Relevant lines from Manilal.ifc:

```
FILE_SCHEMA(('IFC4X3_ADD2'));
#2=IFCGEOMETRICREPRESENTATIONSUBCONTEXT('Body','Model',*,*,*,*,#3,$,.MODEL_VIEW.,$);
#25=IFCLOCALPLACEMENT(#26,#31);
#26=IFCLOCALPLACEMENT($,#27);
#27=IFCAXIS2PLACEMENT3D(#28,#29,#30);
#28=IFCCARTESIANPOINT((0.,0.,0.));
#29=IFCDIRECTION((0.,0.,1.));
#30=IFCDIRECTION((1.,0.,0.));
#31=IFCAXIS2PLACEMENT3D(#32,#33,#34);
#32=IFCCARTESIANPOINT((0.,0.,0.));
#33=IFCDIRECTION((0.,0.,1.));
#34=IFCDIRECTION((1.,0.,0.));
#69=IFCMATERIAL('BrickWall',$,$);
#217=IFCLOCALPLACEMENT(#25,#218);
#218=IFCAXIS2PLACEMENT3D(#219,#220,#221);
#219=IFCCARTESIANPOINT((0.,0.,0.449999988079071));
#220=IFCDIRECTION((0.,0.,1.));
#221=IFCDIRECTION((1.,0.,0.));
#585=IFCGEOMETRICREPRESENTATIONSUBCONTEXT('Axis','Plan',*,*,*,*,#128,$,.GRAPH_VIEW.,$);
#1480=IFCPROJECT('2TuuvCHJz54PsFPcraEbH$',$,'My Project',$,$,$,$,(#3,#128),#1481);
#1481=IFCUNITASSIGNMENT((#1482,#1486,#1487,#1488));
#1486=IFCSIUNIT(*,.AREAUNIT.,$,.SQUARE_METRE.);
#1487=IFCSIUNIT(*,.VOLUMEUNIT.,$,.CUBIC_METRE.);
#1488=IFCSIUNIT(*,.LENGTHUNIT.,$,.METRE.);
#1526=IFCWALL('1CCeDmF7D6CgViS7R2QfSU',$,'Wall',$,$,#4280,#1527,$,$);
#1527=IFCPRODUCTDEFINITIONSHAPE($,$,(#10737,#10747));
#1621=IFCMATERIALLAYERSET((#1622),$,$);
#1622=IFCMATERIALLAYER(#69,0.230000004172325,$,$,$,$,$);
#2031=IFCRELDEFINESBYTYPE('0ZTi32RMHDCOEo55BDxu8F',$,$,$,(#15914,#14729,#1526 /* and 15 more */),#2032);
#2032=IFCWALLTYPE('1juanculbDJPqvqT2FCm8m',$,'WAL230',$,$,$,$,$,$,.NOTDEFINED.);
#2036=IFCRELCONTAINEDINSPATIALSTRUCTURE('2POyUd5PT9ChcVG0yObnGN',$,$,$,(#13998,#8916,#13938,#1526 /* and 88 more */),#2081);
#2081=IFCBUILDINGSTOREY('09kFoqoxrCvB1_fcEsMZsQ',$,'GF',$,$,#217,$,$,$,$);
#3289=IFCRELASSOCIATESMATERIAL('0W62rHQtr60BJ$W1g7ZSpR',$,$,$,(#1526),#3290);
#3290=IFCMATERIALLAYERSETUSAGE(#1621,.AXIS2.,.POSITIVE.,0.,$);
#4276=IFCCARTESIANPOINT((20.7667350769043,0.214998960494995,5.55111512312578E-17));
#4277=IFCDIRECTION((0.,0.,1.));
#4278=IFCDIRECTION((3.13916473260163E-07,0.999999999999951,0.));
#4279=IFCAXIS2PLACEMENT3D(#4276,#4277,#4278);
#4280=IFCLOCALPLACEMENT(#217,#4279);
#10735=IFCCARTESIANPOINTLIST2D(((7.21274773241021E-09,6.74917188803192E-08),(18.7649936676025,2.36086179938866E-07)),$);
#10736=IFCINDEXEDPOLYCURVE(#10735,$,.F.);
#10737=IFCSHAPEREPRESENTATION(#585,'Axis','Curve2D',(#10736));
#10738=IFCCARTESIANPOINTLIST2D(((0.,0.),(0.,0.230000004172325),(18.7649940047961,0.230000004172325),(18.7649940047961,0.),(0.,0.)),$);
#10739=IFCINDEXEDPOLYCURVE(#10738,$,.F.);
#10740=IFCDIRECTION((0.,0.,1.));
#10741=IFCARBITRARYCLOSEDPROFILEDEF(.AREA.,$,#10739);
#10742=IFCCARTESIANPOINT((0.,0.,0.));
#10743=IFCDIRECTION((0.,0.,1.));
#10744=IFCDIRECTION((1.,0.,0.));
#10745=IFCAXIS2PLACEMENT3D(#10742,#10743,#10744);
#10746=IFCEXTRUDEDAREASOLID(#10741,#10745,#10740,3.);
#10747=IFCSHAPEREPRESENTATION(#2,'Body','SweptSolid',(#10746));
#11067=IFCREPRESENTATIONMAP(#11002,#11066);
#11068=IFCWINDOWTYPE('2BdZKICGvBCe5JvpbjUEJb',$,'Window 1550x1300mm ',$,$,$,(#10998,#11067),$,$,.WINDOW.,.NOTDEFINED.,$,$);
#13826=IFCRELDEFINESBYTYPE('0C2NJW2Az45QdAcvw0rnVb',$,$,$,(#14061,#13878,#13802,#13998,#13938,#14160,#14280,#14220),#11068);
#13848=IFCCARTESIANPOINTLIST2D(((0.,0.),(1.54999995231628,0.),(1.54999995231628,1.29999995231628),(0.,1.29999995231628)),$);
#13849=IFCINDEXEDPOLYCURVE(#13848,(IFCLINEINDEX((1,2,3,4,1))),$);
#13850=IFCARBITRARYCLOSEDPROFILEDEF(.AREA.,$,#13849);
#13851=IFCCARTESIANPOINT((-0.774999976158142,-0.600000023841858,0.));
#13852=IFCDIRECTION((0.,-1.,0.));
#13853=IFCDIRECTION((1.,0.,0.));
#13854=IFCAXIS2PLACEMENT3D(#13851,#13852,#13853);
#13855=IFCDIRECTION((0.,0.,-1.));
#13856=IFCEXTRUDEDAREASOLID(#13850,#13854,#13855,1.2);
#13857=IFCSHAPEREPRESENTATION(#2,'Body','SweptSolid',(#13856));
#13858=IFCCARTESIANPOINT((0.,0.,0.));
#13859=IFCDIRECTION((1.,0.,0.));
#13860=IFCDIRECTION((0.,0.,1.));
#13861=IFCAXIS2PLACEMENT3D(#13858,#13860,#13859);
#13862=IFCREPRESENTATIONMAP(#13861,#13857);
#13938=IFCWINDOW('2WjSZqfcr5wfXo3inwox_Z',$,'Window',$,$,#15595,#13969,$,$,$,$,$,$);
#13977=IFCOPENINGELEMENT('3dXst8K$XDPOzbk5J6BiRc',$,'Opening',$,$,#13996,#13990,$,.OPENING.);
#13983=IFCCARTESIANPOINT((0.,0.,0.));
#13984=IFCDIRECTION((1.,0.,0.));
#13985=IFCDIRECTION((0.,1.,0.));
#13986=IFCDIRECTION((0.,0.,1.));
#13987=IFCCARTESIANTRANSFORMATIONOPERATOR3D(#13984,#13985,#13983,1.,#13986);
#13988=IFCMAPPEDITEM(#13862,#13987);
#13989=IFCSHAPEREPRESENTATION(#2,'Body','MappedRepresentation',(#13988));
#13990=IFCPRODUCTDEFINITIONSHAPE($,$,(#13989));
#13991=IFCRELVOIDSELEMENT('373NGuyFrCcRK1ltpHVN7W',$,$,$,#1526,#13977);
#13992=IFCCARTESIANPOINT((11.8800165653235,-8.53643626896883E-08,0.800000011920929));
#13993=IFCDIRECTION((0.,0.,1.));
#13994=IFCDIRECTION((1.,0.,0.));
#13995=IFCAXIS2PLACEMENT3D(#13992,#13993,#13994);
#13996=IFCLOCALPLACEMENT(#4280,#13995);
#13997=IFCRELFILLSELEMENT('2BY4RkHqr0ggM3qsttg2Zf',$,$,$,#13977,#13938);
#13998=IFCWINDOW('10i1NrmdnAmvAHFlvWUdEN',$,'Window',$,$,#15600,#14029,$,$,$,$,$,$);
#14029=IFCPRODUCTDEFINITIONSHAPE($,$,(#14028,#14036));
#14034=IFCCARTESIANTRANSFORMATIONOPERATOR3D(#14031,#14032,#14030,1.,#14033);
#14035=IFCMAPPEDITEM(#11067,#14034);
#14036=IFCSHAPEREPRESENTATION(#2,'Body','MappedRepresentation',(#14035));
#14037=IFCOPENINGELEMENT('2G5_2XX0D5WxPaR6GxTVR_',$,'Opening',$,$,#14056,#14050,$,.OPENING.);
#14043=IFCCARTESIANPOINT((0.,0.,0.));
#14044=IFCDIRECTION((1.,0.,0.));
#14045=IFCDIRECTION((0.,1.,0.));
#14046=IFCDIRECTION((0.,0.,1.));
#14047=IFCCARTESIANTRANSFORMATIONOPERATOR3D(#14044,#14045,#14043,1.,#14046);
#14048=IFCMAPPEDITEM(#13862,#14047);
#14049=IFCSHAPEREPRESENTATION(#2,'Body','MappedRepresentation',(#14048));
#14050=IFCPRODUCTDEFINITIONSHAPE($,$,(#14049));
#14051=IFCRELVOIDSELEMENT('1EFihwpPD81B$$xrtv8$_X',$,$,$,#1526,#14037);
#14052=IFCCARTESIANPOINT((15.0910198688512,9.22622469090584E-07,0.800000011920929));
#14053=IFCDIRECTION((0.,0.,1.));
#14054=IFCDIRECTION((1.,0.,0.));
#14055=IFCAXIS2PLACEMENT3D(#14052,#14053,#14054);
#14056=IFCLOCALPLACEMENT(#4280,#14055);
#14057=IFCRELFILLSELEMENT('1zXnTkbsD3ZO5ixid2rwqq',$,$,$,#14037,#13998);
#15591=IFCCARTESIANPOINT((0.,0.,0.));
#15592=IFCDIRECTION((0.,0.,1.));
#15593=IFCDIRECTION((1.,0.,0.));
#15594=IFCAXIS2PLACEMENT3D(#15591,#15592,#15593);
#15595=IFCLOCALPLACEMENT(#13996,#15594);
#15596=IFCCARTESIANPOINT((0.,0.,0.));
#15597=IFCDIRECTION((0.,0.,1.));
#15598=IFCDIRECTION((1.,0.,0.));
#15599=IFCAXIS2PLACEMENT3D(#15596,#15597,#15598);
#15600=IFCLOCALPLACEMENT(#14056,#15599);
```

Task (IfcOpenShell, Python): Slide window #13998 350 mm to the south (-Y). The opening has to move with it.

```python
import ifcopenshell
import ifcopenshell.api.geometry
import ifcopenshell.util.placement
import ifcopenshell.util.unit

model = ifcopenshell.open("Manilal.ifc")
unit_scale = ifcopenshell.util.unit.calculate_unit_scale(model)

window = model.by_guid("10i1NrmdnAmvAHFlvWUdEN")
opening = window.FillsVoids[0].RelatingOpeningElement
wall = opening.VoidsElements[0].RelatingBuildingElement

wall_matrix = ifcopenshell.util.placement.get_local_placement(wall.ObjectPlacement)
shift = wall_matrix[:3, 0] * -0.35 / unit_scale
before = ifcopenshell.util.placement.get_local_placement(window.ObjectPlacement)[:3, 3].copy()

# The window is placed relative to its opening, so it follows when the opening moves.
matrix = ifcopenshell.util.placement.get_local_placement(opening.ObjectPlacement)
matrix[:3, 3] += shift
ifcopenshell.api.geometry.edit_object_placement(
    model, product=opening, matrix=matrix, is_si=False, should_transform_children=True
)

after = ifcopenshell.util.placement.get_local_placement(window.ObjectPlacement)[:3, 3]
print("window moved by", (after - before).round(3) + 0.0)

model.write("Manilal_v2.ifc")
```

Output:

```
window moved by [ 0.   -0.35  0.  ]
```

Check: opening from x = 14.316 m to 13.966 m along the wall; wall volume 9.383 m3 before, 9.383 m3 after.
